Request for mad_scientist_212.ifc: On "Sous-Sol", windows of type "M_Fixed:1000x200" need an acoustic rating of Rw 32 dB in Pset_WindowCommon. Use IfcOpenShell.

First a look at what the model holds.

```python
import ifcopenshell
import ifcopenshell.util.element

model = ifcopenshell.open("mad_scientist_212.ifc")
print(model.schema)
storey = next(s for s in model.by_type("IfcBuildingStorey") if s.Name == "Sous-Sol")
windows = [e for e in ifcopenshell.util.element.get_decomposition(storey) if e.is_a("IfcWindow")]
seen = {}
for e in windows:
    element_type = ifcopenshell.util.element.get_type(e)
    key = (element_type.Name if element_type != e and element_type else None, ifcopenshell.util.element.get_pset(e, "Pset_WindowCommon", "AcousticRating"))
    seen[key] = seen.get(key, 0) + 1
for (name, value), count in sorted(seen.items(), key=str):
    print(count, "x", name, "|", value)
```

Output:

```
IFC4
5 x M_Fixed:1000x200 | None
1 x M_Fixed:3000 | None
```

```python
import ifcopenshell
import ifcopenshell.api.pset
import ifcopenshell.util.element

model = ifcopenshell.open("mad_scientist_212.ifc")

storey = next(s for s in model.by_type("IfcBuildingStorey") if s.Name == "Sous-Sol")
windows = [e for e in ifcopenshell.util.element.get_decomposition(storey) if e.is_a("IfcWindow")]

count = 0
for e in windows:
    element_type = ifcopenshell.util.element.get_type(e)
    if element_type in (None, e) or element_type.Name != "M_Fixed:1000x200":
        continue
    # add_pset returns the element's existing set when there is one.
    pset = ifcopenshell.api.pset.add_pset(model, product=e, name="Pset_WindowCommon")
    ifcopenshell.api.pset.edit_pset(model, pset=pset, properties={"AcousticRating": "Rw 32 dB"})
    count += 1

print(count, "windows updated")

model.write("mad_scientist_212-out.ifc")
```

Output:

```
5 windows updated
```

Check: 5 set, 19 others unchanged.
